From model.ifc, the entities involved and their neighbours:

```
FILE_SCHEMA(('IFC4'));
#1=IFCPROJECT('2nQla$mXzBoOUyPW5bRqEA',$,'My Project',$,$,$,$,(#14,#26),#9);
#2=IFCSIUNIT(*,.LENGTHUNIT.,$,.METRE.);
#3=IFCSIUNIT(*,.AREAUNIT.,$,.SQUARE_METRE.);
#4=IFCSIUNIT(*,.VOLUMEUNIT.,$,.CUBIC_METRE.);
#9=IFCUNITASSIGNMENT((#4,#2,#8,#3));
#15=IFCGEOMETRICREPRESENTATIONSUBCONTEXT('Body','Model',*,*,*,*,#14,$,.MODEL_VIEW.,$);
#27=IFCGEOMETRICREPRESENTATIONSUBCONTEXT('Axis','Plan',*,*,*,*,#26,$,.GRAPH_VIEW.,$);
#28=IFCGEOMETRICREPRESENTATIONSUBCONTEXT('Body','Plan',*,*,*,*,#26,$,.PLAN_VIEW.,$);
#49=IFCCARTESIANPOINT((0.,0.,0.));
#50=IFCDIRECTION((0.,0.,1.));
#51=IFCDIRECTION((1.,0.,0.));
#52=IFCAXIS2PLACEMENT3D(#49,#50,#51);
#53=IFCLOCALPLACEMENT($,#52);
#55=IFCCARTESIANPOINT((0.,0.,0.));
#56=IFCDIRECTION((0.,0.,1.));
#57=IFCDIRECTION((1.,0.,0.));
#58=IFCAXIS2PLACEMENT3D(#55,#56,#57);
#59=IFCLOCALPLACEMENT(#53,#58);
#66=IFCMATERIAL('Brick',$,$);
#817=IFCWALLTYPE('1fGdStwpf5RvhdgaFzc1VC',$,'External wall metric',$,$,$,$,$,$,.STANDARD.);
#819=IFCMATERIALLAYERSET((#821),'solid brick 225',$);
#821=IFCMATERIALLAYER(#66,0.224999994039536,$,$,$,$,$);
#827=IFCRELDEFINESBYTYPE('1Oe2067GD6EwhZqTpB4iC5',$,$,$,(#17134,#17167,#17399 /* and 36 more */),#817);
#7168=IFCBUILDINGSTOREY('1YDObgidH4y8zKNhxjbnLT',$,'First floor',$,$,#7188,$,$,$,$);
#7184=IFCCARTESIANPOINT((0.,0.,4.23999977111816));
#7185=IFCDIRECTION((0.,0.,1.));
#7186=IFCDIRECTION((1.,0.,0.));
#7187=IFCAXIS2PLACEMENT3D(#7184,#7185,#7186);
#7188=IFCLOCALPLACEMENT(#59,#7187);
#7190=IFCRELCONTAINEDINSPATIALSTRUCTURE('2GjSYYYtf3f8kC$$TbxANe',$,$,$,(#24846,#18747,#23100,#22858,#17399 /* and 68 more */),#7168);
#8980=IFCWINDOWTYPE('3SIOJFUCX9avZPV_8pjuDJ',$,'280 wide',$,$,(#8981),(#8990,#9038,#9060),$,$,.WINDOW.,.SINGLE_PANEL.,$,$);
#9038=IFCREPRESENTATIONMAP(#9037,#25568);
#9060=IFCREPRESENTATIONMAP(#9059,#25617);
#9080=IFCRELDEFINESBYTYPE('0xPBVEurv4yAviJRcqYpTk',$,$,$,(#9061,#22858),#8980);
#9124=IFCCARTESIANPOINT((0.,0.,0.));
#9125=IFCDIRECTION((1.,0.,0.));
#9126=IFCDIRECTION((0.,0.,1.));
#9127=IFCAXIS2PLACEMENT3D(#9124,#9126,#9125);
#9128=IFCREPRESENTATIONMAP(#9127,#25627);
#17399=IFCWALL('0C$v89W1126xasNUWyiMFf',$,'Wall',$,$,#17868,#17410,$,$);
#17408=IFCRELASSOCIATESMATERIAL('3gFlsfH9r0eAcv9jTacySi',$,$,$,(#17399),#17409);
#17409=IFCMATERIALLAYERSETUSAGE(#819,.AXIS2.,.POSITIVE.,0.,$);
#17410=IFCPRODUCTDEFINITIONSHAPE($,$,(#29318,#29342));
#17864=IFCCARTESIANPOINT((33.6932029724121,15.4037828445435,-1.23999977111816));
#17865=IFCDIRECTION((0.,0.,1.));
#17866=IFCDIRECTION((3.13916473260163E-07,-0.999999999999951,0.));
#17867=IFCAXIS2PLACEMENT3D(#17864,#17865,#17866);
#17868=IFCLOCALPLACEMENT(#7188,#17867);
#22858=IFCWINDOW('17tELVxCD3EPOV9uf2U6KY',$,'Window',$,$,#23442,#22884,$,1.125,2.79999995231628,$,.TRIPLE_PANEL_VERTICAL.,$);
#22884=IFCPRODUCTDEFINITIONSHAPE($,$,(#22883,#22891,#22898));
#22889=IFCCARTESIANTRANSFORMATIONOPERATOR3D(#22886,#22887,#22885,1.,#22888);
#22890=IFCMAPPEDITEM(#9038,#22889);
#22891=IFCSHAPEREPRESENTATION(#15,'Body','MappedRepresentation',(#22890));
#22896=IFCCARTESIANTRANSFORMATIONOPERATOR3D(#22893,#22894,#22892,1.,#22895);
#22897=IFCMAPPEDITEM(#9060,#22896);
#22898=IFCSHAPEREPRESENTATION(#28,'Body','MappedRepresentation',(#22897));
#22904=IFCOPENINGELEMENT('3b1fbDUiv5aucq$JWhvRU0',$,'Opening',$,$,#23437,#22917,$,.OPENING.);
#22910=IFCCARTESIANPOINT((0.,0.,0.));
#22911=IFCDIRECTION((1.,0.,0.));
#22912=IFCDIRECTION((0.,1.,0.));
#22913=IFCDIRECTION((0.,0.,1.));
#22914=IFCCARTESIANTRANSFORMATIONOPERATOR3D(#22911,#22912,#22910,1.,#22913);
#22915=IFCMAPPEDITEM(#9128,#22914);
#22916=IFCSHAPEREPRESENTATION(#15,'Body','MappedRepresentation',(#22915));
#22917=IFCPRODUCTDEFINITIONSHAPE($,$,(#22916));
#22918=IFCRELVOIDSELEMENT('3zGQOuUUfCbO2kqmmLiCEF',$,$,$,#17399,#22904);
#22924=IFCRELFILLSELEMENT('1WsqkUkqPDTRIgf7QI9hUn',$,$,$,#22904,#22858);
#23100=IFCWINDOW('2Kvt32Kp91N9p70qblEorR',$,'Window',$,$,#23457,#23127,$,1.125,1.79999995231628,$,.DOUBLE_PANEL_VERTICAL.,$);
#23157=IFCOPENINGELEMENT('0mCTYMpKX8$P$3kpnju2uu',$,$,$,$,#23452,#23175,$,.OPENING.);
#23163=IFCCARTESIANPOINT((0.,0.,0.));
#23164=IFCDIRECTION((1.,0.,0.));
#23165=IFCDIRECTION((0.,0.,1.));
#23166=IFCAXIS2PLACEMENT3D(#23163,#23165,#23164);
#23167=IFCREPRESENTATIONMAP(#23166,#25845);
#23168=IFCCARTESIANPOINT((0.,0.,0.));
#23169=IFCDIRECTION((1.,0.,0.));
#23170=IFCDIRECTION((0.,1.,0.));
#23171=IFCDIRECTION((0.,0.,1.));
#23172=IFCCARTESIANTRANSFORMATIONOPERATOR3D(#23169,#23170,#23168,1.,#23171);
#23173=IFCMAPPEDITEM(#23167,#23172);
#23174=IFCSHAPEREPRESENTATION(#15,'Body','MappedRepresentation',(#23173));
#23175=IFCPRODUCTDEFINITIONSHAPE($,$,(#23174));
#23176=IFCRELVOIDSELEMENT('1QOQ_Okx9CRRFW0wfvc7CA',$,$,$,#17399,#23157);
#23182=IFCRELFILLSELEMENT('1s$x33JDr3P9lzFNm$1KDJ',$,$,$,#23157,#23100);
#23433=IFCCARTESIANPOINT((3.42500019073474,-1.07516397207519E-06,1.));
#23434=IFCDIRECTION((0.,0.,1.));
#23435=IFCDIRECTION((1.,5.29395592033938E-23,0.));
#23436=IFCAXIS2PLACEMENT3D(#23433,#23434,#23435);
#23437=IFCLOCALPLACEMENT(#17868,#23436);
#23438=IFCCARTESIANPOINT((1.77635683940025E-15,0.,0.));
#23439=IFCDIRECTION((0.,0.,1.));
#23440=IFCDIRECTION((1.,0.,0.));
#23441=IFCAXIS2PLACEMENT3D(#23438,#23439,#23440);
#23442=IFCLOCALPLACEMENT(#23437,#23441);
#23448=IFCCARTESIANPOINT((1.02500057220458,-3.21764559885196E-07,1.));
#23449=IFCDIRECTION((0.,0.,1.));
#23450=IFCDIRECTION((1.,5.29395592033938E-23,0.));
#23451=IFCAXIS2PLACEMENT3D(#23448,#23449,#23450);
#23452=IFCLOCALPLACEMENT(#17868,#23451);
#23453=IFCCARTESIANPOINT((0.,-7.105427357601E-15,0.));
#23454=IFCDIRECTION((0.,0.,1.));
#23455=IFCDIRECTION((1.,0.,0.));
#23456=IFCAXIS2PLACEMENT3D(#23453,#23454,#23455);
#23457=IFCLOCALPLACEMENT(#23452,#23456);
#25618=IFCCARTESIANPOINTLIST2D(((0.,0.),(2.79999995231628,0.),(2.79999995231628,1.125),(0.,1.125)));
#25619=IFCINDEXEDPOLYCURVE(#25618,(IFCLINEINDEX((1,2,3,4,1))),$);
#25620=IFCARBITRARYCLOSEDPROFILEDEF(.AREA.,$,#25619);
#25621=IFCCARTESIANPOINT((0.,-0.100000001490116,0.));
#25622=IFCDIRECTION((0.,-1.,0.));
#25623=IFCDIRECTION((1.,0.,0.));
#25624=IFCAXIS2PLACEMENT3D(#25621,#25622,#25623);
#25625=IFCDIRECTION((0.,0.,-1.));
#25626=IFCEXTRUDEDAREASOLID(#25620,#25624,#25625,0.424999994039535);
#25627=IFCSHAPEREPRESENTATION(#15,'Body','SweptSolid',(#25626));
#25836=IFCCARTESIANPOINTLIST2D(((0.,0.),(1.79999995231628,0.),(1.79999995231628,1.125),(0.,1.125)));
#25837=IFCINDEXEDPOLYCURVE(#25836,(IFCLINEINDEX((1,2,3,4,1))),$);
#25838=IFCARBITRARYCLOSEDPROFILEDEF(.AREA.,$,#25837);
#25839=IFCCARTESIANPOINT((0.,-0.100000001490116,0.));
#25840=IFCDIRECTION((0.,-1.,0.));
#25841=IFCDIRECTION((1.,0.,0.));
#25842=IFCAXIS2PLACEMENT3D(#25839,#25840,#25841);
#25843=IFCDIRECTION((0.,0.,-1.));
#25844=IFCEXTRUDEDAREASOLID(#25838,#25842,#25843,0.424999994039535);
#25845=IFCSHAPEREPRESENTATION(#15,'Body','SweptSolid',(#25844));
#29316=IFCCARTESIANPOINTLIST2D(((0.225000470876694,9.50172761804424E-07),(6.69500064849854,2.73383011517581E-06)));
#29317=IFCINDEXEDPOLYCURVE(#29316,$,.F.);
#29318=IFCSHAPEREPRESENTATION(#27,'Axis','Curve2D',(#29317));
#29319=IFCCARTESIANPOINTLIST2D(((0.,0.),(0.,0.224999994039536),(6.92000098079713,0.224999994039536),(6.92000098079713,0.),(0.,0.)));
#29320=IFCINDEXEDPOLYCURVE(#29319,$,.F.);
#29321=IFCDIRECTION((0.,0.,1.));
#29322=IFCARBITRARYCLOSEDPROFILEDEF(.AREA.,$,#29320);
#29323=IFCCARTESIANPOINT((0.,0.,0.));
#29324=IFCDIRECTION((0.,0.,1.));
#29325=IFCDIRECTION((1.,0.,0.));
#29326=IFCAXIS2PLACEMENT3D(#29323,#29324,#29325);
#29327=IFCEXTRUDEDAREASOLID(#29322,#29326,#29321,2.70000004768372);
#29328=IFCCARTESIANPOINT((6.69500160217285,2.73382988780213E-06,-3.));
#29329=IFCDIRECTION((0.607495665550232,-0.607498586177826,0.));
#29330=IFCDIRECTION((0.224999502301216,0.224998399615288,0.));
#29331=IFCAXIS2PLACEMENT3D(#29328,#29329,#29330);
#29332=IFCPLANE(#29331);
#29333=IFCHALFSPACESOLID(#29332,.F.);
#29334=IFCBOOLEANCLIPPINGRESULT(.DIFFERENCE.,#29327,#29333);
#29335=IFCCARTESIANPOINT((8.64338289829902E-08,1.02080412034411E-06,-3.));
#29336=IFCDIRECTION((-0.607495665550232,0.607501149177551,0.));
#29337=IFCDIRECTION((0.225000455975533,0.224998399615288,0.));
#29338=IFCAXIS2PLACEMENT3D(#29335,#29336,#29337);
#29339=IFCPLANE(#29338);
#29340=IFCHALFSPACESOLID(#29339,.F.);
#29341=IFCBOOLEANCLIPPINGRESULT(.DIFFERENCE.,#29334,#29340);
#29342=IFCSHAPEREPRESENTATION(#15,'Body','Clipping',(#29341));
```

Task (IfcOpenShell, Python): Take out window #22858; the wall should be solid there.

```python
import ifcopenshell
import ifcopenshell.api.feature
import ifcopenshell.api.root
import ifcopenshell.geom
import ifcopenshell.util.shape

model = ifcopenshell.open("model.ifc")
settings = ifcopenshell.geom.settings()


def volume(element):
    """Net volume in cubic metres, openings subtracted."""
    shape = ifcopenshell.geom.create_shape(settings, element)
    return ifcopenshell.util.shape.get_volume(shape.geometry)


window = model.by_guid("17tELVxCD3EPOV9uf2U6KY")
opening = window.FillsVoids[0].RelatingOpeningElement
wall = opening.VoidsElements[0].RelatingBuildingElement
before = volume(wall)

ifcopenshell.api.root.remove_product(model, product=window)
ifcopenshell.api.feature.remove_feature(model, feature=opening)

after = volume(wall)

print(f"wall volume {before:.3f} -> {after:.3f} m3")

model.write("model-out.ifc")
```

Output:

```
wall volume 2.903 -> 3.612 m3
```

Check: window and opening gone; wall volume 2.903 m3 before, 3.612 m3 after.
